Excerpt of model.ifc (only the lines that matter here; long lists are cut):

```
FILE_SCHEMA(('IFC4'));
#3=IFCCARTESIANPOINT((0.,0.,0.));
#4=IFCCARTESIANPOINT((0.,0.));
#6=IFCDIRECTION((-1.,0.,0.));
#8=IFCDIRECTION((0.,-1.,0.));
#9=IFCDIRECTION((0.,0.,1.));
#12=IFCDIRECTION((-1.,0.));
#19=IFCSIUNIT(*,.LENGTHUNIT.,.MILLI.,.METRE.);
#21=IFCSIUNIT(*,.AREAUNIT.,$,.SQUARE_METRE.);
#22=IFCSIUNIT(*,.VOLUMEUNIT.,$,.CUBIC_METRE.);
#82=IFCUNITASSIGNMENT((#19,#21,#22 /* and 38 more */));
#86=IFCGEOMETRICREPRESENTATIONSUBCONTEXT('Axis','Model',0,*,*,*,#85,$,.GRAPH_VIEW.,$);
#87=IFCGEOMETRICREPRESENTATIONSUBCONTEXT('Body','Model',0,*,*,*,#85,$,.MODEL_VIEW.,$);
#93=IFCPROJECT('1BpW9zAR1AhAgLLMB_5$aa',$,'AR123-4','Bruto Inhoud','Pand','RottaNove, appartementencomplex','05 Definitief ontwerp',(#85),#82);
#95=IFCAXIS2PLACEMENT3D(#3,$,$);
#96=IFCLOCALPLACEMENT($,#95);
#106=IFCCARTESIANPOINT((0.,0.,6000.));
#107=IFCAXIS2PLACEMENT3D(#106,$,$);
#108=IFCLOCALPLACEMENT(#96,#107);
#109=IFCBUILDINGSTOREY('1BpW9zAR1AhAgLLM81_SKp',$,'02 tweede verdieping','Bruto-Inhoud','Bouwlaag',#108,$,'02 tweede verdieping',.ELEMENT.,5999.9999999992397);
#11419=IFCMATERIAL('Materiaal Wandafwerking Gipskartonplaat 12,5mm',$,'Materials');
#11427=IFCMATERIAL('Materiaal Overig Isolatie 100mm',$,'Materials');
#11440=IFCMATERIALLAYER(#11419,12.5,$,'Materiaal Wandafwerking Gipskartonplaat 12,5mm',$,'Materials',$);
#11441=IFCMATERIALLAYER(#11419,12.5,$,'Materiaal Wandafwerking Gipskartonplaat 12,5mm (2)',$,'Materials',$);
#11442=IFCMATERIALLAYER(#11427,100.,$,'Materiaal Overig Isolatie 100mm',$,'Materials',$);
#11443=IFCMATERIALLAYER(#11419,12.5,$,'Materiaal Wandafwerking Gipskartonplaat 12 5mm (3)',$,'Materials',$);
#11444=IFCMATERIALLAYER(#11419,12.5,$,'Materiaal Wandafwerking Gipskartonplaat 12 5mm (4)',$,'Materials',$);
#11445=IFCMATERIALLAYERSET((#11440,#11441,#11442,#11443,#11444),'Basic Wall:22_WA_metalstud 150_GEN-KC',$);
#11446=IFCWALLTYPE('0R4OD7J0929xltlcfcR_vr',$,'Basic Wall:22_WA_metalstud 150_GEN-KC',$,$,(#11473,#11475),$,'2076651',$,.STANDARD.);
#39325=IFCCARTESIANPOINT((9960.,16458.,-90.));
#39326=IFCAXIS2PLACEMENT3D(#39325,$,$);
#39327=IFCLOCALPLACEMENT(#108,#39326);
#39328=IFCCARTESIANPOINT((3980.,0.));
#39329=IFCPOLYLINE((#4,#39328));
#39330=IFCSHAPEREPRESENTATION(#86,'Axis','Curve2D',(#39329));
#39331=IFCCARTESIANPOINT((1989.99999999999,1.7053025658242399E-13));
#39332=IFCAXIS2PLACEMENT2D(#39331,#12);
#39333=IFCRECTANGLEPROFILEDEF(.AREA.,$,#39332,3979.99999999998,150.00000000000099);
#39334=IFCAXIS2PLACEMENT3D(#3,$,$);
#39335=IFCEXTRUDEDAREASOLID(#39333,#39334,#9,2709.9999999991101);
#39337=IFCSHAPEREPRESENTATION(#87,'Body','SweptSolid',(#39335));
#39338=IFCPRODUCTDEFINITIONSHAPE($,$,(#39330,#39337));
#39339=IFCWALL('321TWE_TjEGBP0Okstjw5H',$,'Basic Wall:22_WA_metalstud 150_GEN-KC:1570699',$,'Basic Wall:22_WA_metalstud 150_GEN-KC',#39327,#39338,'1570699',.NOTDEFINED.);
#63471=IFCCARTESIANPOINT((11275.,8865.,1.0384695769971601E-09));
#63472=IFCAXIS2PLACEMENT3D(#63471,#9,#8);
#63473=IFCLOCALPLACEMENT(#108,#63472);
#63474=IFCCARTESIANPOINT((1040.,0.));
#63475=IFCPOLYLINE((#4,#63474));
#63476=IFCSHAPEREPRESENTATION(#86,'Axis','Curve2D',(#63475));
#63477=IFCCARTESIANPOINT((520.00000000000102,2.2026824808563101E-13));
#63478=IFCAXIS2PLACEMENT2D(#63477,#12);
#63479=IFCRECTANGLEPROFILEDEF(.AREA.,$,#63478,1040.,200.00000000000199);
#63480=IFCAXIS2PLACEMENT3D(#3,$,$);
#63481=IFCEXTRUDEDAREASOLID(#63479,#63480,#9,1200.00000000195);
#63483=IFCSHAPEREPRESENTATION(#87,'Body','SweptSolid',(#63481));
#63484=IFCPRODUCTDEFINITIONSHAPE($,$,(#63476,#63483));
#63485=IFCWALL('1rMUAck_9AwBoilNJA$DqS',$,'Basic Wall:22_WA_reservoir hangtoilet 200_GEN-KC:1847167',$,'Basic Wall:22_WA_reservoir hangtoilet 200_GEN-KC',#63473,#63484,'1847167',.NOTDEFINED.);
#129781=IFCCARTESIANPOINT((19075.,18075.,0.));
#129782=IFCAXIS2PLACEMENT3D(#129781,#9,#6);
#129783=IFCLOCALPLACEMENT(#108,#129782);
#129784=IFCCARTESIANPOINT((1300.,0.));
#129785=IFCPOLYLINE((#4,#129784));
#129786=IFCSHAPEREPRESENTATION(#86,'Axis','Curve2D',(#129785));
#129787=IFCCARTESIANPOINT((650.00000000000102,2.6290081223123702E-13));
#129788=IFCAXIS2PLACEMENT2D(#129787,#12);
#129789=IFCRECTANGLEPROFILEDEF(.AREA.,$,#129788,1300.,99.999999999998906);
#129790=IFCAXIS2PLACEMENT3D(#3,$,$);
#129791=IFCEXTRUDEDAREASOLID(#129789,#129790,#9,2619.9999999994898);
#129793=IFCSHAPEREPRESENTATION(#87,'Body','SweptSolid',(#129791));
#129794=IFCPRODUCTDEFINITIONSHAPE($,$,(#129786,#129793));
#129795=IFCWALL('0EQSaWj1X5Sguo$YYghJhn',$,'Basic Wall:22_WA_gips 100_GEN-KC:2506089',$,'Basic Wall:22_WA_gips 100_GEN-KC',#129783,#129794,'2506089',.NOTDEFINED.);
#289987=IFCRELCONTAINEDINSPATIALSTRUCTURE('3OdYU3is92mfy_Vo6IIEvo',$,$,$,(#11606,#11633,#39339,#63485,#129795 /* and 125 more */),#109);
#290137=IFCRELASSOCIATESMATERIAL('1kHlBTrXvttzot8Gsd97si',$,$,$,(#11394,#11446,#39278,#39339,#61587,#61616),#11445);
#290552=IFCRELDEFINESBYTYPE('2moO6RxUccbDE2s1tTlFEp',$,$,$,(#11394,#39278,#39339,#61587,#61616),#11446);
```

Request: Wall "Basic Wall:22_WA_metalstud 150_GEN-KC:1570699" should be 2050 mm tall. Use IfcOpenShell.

```python
import ifcopenshell
import ifcopenshell.geom
import ifcopenshell.util.representation
import ifcopenshell.util.shape

model = ifcopenshell.open("model.ifc")
settings = ifcopenshell.geom.settings()


def volume(element):
    """Net volume in cubic metres, openings subtracted."""
    shape = ifcopenshell.geom.create_shape(settings, element)
    return ifcopenshell.util.shape.get_volume(shape.geometry)


wall = model.by_guid("321TWE_TjEGBP0Okstjw5H")
before = volume(wall)

body = ifcopenshell.util.representation.get_representation(wall, "Model", "Body")
solid = body.Items[0]
old_height = solid.Depth
solid.Depth = 2050.0
after = volume(wall)

print(f"height {old_height:g} -> {solid.Depth:g}, volume {before:.3f} -> {after:.3f} m3")

model.write("model_edited.ifc")
```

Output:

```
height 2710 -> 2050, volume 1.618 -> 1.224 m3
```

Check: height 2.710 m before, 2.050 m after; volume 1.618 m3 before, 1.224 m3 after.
